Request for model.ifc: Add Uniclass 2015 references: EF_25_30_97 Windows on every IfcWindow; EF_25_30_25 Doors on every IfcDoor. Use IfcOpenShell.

First a look at what the model holds.

```python
import ifcopenshell

model = ifcopenshell.open("model.ifc")
print(model.schema)
print("classifications:", [c.Name for c in model.by_type("IfcClassification")])
for ifc_class in ("IfcDoor", "IfcRoof", "IfcStair", "IfcWall", "IfcWindow"):
    print(ifc_class, len(model.by_type(ifc_class)))
```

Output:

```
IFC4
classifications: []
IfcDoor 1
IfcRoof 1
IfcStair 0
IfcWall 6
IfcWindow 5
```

```python
import ifcopenshell
import ifcopenshell.api.classification

model = ifcopenshell.open("model.ifc")

system = ifcopenshell.api.classification.add_classification(model, classification="Uniclass 2015")

codes = {
    "IfcWindow": ("EF_25_30_97", "Windows"),
    "IfcDoor": ("EF_25_30_25", "Doors"),
}
for ifc_class, (code, name) in codes.items():
    products = model.by_type(ifc_class)
    ifcopenshell.api.classification.add_reference(
        model, products=products, classification=system, identification=code, name=name
    )
    print(code, len(products))

model.write("model_updated.ifc")
```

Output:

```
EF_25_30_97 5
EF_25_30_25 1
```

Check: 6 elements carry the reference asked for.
